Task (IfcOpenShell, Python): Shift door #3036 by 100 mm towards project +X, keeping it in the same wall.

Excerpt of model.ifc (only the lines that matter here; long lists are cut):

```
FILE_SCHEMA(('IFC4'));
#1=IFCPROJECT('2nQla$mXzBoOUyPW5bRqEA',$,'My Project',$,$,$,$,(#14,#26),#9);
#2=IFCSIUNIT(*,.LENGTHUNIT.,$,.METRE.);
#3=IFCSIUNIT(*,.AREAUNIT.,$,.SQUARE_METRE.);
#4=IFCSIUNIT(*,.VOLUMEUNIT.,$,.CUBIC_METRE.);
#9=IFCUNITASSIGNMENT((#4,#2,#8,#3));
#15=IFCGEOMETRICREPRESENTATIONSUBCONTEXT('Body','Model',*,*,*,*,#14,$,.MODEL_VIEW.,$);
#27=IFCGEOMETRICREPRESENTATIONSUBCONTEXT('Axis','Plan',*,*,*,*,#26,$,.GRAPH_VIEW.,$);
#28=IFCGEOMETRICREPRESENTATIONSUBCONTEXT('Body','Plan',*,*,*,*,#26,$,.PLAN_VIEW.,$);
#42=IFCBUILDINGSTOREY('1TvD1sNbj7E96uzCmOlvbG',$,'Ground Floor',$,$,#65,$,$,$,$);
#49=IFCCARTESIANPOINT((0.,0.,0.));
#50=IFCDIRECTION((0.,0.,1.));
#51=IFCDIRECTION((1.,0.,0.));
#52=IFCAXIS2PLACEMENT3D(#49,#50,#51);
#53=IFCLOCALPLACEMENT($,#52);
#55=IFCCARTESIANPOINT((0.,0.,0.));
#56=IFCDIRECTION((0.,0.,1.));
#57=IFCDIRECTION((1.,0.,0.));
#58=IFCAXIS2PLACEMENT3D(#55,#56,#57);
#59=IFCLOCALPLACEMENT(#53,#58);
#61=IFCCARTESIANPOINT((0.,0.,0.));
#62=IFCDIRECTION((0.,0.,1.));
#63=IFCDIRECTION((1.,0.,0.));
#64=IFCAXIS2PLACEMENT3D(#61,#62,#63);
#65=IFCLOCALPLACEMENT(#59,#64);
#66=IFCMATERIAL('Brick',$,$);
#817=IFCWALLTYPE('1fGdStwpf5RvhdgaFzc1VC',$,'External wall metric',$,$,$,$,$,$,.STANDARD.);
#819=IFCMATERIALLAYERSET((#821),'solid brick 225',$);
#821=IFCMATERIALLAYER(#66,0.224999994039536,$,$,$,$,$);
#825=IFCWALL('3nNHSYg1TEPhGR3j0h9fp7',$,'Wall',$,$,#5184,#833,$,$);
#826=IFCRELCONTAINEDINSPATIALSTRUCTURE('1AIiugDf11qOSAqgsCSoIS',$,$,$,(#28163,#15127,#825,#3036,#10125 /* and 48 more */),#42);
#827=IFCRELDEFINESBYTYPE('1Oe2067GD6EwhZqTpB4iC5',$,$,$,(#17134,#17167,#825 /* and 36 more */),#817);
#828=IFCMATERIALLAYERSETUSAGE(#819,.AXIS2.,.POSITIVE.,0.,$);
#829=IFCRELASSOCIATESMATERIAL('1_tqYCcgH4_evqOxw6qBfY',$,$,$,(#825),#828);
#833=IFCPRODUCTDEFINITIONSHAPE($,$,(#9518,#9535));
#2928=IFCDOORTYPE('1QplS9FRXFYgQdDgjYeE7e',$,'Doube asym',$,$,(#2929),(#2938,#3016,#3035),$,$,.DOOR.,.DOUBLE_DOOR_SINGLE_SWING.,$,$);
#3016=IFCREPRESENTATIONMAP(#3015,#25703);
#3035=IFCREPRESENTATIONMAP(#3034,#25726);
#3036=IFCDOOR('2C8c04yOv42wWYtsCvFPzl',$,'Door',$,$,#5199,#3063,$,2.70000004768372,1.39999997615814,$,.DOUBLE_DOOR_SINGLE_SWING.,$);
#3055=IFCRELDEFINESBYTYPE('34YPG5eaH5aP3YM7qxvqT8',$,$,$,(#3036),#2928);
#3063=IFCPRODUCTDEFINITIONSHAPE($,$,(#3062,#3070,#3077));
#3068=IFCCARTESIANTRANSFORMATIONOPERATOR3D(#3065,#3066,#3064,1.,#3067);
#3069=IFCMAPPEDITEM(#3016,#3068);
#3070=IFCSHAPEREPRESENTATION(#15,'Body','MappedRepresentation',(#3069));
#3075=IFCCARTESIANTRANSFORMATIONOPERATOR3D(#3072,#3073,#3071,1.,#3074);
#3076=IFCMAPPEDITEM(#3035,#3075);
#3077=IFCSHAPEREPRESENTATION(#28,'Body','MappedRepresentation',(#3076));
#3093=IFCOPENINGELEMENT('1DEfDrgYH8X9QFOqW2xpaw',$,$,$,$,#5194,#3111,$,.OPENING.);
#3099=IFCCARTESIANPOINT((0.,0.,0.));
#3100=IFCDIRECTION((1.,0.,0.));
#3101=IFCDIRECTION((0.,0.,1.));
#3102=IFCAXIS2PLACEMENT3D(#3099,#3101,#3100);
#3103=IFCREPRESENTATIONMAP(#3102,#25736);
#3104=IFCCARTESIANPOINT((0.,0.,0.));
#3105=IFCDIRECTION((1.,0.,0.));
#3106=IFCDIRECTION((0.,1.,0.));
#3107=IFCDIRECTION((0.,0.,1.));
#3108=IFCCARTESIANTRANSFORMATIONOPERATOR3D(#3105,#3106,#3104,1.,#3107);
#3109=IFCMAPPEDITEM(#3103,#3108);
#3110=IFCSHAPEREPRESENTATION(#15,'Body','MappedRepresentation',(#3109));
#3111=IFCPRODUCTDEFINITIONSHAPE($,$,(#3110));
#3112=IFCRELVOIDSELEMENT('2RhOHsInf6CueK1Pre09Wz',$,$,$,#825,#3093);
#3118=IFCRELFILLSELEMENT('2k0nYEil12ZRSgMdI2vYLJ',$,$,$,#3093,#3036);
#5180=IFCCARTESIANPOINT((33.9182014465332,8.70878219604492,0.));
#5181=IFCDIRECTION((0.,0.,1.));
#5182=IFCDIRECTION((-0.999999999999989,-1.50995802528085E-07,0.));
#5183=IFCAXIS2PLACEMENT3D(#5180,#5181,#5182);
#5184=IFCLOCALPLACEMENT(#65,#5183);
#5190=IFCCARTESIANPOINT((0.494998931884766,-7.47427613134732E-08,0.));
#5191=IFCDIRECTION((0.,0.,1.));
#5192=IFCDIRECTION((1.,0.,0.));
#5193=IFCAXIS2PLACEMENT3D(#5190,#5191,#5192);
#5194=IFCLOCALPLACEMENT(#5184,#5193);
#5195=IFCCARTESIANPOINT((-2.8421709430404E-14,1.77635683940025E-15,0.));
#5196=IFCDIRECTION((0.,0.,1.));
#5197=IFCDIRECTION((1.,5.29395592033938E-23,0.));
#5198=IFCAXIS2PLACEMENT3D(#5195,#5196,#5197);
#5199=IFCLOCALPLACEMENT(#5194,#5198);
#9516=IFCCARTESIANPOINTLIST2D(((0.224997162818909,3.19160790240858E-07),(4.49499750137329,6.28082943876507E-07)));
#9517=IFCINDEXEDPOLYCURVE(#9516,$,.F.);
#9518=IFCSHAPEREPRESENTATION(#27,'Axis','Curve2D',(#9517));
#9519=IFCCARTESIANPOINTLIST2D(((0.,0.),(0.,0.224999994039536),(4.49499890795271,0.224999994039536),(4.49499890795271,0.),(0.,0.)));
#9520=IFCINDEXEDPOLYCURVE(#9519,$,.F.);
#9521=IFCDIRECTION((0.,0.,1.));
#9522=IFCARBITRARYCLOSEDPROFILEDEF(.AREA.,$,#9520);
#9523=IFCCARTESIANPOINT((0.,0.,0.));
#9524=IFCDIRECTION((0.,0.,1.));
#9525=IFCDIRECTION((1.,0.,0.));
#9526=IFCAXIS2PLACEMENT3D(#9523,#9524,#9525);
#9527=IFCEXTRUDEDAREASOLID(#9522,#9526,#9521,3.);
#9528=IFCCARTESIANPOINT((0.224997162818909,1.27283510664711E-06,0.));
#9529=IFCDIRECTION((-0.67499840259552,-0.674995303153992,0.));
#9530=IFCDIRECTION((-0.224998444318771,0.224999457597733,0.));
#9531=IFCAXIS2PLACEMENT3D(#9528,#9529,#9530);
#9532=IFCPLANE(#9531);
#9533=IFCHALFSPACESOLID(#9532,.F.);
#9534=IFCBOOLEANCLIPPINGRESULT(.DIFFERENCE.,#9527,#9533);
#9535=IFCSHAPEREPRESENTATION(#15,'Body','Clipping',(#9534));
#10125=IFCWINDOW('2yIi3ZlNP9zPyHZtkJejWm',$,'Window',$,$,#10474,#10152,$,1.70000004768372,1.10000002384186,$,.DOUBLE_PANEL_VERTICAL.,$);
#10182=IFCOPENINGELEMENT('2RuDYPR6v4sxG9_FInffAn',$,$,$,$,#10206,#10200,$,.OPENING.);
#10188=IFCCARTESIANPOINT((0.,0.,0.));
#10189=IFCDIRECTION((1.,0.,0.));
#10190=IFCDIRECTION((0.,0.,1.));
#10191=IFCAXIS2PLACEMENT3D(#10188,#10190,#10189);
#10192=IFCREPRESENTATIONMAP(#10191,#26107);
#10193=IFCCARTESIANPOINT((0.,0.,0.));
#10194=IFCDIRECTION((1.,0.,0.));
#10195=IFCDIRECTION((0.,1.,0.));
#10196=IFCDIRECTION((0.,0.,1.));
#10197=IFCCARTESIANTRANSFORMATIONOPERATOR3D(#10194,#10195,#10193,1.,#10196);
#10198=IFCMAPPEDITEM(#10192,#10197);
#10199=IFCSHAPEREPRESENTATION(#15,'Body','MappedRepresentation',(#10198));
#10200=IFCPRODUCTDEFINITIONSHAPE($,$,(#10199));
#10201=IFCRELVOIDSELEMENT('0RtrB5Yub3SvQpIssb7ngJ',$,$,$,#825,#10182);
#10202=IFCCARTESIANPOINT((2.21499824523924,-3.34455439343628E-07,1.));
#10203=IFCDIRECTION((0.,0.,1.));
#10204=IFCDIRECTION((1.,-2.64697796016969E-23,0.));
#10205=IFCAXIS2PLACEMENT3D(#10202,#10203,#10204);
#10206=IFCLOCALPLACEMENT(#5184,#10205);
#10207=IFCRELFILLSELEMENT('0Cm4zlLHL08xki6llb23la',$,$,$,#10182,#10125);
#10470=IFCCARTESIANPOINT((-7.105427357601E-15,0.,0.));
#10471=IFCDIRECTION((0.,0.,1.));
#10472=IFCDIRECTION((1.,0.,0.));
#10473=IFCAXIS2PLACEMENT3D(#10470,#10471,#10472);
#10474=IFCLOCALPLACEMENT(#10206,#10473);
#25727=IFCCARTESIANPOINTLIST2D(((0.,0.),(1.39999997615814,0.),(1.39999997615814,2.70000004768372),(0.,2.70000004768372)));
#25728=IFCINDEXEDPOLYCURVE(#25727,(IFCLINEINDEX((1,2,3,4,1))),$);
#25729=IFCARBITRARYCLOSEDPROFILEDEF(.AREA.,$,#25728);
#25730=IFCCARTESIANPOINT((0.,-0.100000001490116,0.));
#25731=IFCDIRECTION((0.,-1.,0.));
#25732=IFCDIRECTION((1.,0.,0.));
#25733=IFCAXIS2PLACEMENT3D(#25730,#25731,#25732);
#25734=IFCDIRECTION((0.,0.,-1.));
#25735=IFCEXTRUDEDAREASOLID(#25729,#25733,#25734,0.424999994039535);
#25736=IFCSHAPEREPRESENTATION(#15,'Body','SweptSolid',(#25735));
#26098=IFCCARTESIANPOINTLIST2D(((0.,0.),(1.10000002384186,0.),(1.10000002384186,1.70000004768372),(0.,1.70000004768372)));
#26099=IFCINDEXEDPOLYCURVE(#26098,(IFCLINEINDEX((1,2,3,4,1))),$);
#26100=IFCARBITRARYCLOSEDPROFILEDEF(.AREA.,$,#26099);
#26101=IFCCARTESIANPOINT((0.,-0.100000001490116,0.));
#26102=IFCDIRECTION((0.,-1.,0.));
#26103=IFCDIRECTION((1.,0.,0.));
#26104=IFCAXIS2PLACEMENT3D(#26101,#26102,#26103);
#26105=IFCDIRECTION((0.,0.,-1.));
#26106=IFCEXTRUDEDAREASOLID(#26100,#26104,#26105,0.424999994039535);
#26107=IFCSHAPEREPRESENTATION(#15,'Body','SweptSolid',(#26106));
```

```python
import ifcopenshell
import ifcopenshell.api.geometry
import ifcopenshell.util.placement
import ifcopenshell.util.unit

model = ifcopenshell.open("model.ifc")
unit_scale = ifcopenshell.util.unit.calculate_unit_scale(model)

door = model.by_id(3036)
opening = door.FillsVoids[0].RelatingOpeningElement
wall = opening.VoidsElements[0].RelatingBuildingElement

wall_matrix = ifcopenshell.util.placement.get_local_placement(wall.ObjectPlacement)
shift = wall_matrix[:3, 0] * -0.1 / unit_scale
before = ifcopenshell.util.placement.get_local_placement(door.ObjectPlacement)[:3, 3].copy()

# The door is placed relative to its opening, so it follows when the opening moves.
matrix = ifcopenshell.util.placement.get_local_placement(opening.ObjectPlacement)
matrix[:3, 3] += shift
ifcopenshell.api.geometry.edit_object_placement(
    model, product=opening, matrix=matrix, is_si=False, should_transform_children=True
)

after = ifcopenshell.util.placement.get_local_placement(door.ObjectPlacement)[:3, 3]
print("door moved by", (after - before).round(3) + 0.0)

model.write("model_updated.ifc")
```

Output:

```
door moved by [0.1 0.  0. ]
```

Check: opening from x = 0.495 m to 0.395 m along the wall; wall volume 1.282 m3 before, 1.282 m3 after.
